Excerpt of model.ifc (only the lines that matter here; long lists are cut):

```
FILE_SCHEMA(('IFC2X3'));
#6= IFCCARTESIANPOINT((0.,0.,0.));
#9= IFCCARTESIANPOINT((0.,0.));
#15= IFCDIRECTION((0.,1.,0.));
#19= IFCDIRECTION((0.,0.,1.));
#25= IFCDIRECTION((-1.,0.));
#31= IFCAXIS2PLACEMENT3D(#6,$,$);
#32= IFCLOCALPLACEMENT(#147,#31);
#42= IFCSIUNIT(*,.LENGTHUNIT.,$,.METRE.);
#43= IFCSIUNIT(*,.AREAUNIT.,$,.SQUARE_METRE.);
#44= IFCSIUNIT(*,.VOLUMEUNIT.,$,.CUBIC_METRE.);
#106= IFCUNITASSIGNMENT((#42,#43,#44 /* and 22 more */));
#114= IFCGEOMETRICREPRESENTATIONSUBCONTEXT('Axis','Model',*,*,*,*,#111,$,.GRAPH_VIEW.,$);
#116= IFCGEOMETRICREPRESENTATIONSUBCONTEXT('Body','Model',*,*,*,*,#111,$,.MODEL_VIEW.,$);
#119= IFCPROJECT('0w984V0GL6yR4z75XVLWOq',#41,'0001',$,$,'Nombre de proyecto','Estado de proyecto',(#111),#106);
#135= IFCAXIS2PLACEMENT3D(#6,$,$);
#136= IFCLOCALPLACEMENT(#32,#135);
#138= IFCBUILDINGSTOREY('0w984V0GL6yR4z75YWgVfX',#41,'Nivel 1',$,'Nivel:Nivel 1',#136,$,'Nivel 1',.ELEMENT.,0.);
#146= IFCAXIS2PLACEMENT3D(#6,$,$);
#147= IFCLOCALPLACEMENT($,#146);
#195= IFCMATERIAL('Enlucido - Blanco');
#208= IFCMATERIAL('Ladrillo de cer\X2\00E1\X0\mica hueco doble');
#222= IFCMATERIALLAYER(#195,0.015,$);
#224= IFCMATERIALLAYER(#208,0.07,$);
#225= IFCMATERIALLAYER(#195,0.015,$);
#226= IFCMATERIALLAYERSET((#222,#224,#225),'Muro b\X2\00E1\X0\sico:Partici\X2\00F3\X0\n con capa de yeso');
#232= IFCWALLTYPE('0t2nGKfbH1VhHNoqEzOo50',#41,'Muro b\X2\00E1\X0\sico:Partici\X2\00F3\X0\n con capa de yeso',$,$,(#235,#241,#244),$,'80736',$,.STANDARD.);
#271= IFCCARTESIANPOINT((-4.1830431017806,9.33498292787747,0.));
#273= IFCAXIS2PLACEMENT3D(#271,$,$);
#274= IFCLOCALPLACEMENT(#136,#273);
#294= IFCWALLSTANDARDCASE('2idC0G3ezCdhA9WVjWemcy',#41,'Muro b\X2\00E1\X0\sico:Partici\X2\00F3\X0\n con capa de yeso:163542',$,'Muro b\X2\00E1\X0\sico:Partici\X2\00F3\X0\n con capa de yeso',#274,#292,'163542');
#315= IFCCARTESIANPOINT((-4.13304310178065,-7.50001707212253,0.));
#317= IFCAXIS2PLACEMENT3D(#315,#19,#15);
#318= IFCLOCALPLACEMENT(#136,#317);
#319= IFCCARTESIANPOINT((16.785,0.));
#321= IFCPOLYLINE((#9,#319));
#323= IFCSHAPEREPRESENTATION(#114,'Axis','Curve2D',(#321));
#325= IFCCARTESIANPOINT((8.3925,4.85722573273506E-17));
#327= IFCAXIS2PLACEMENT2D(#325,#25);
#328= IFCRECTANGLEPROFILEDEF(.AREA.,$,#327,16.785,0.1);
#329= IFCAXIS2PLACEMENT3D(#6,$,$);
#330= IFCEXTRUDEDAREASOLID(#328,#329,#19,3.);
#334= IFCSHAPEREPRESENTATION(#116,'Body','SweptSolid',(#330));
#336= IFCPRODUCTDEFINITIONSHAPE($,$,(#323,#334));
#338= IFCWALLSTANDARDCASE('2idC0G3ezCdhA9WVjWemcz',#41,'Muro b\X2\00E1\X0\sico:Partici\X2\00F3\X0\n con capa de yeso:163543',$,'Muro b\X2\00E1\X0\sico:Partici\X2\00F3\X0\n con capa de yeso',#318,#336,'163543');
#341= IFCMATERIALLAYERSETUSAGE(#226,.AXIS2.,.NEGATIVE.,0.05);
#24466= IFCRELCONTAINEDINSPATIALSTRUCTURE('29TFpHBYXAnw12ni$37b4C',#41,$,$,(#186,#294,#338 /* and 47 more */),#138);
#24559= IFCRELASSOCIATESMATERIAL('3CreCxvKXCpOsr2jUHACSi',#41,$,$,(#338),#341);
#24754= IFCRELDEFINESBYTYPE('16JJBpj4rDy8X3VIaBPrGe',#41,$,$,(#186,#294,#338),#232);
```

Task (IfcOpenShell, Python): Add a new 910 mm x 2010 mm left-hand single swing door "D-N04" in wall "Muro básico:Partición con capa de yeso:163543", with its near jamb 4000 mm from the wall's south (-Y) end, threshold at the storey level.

```python
import numpy as np
import ifcopenshell
import ifcopenshell.api.feature
import ifcopenshell.api.geometry
import ifcopenshell.api.root
import ifcopenshell.api.spatial
import ifcopenshell.api.type
import ifcopenshell.geom
import ifcopenshell.util.element
import ifcopenshell.util.placement
import ifcopenshell.util.representation
import ifcopenshell.util.shape
import ifcopenshell.util.unit

model = ifcopenshell.open("model.ifc")
unit_scale = ifcopenshell.util.unit.calculate_unit_scale(model)
settings = ifcopenshell.geom.settings()


def volume(element):
    """Net volume in cubic metres, openings subtracted."""
    shape = ifcopenshell.geom.create_shape(settings, element)
    return ifcopenshell.util.shape.get_volume(shape.geometry)


wall = model.by_guid("2idC0G3ezCdhA9WVjWemcz")
storey = ifcopenshell.util.element.get_container(wall, ifc_class="IfcBuildingStorey")
context = ifcopenshell.util.representation.get_context(model, "Model", "Body", "MODEL_VIEW")
before = volume(wall)

width, height, from_end, sill = 0.91, 2.01, 4, 0.0  # metres

# The wall runs along its own X axis, and the end named is its -X end.
wall_shape = ifcopenshell.geom.create_shape(settings, wall)
x, y, z = ifcopenshell.util.shape.get_vertices(wall_shape.geometry).T
start = x.min() + from_end
face, thickness = float(y.min()), float(y.max() - y.min())
wall_matrix = ifcopenshell.util.placement.get_local_placement(wall.ObjectPlacement)
level = ifcopenshell.util.placement.get_local_placement(storey.ObjectPlacement)[2, 3]


def in_wall(x, y):
    """Placement at x, y metres in the wall's axes, at sill height."""
    matrix = wall_matrix.copy()
    matrix[:, 3] = wall_matrix @ np.array([x / unit_scale, y / unit_scale, 0.0, 1.0])
    matrix[2, 3] = level + sill / unit_scale
    return matrix


# Opening: a box that overshoots both wall faces by 50 mm.
opening = ifcopenshell.api.root.create_entity(model, ifc_class="IfcOpeningElement")
box = ifcopenshell.api.geometry.add_wall_representation(
    model, context=context, length=width, height=height, thickness=thickness + 0.1
)
ifcopenshell.api.geometry.assign_representation(model, product=opening, representation=box)
ifcopenshell.api.geometry.edit_object_placement(model, product=opening, matrix=in_wall(start, face - 0.05), is_si=False)
ifcopenshell.api.feature.add_feature(model, feature=opening, element=wall)

door = ifcopenshell.api.root.create_entity(model, ifc_class="IfcDoor", name="D-N04")
door.OverallWidth, door.OverallHeight = width / unit_scale, height / unit_scale
body = ifcopenshell.api.geometry.add_door_representation(
    model,
    context=context,
    overall_width=door.OverallWidth,
    overall_height=door.OverallHeight,
    operation_type="SINGLE_SWING_LEFT",
    lining_properties={"LiningDepth": thickness / unit_scale, "ThresholdDepth": thickness / unit_scale},
)
ifcopenshell.api.geometry.assign_representation(model, product=door, representation=body)
ifcopenshell.api.spatial.assign_container(model, products=[door], relating_structure=storey)
fills = ifcopenshell.api.feature.add_filling(model, opening=opening, element=door)
fills.OwnerHistory = door.OwnerHistory  # required in IFC2X3

# IFC2X3 keeps the operation on the door style.
style = ifcopenshell.api.root.create_entity(model, ifc_class="IfcDoorStyle", name="D-N04")
style.OperationType, style.ConstructionType = "SINGLE_SWING_LEFT", "NOTDEFINED"
style.ParameterTakesPrecedence = style.Sizeable = False
ifcopenshell.api.type.assign_type(model, related_objects=[door], relating_type=style)

# The lining spans the wall, so the door starts at the wall face.
ifcopenshell.api.geometry.edit_object_placement(model, product=door, matrix=in_wall(start, face), is_si=False)

after = volume(wall)

print(f"wall volume {before:.3f} -> {after:.3f} m3")

model.write("model-out.ifc")
```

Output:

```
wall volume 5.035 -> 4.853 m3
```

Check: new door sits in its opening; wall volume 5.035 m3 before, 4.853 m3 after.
